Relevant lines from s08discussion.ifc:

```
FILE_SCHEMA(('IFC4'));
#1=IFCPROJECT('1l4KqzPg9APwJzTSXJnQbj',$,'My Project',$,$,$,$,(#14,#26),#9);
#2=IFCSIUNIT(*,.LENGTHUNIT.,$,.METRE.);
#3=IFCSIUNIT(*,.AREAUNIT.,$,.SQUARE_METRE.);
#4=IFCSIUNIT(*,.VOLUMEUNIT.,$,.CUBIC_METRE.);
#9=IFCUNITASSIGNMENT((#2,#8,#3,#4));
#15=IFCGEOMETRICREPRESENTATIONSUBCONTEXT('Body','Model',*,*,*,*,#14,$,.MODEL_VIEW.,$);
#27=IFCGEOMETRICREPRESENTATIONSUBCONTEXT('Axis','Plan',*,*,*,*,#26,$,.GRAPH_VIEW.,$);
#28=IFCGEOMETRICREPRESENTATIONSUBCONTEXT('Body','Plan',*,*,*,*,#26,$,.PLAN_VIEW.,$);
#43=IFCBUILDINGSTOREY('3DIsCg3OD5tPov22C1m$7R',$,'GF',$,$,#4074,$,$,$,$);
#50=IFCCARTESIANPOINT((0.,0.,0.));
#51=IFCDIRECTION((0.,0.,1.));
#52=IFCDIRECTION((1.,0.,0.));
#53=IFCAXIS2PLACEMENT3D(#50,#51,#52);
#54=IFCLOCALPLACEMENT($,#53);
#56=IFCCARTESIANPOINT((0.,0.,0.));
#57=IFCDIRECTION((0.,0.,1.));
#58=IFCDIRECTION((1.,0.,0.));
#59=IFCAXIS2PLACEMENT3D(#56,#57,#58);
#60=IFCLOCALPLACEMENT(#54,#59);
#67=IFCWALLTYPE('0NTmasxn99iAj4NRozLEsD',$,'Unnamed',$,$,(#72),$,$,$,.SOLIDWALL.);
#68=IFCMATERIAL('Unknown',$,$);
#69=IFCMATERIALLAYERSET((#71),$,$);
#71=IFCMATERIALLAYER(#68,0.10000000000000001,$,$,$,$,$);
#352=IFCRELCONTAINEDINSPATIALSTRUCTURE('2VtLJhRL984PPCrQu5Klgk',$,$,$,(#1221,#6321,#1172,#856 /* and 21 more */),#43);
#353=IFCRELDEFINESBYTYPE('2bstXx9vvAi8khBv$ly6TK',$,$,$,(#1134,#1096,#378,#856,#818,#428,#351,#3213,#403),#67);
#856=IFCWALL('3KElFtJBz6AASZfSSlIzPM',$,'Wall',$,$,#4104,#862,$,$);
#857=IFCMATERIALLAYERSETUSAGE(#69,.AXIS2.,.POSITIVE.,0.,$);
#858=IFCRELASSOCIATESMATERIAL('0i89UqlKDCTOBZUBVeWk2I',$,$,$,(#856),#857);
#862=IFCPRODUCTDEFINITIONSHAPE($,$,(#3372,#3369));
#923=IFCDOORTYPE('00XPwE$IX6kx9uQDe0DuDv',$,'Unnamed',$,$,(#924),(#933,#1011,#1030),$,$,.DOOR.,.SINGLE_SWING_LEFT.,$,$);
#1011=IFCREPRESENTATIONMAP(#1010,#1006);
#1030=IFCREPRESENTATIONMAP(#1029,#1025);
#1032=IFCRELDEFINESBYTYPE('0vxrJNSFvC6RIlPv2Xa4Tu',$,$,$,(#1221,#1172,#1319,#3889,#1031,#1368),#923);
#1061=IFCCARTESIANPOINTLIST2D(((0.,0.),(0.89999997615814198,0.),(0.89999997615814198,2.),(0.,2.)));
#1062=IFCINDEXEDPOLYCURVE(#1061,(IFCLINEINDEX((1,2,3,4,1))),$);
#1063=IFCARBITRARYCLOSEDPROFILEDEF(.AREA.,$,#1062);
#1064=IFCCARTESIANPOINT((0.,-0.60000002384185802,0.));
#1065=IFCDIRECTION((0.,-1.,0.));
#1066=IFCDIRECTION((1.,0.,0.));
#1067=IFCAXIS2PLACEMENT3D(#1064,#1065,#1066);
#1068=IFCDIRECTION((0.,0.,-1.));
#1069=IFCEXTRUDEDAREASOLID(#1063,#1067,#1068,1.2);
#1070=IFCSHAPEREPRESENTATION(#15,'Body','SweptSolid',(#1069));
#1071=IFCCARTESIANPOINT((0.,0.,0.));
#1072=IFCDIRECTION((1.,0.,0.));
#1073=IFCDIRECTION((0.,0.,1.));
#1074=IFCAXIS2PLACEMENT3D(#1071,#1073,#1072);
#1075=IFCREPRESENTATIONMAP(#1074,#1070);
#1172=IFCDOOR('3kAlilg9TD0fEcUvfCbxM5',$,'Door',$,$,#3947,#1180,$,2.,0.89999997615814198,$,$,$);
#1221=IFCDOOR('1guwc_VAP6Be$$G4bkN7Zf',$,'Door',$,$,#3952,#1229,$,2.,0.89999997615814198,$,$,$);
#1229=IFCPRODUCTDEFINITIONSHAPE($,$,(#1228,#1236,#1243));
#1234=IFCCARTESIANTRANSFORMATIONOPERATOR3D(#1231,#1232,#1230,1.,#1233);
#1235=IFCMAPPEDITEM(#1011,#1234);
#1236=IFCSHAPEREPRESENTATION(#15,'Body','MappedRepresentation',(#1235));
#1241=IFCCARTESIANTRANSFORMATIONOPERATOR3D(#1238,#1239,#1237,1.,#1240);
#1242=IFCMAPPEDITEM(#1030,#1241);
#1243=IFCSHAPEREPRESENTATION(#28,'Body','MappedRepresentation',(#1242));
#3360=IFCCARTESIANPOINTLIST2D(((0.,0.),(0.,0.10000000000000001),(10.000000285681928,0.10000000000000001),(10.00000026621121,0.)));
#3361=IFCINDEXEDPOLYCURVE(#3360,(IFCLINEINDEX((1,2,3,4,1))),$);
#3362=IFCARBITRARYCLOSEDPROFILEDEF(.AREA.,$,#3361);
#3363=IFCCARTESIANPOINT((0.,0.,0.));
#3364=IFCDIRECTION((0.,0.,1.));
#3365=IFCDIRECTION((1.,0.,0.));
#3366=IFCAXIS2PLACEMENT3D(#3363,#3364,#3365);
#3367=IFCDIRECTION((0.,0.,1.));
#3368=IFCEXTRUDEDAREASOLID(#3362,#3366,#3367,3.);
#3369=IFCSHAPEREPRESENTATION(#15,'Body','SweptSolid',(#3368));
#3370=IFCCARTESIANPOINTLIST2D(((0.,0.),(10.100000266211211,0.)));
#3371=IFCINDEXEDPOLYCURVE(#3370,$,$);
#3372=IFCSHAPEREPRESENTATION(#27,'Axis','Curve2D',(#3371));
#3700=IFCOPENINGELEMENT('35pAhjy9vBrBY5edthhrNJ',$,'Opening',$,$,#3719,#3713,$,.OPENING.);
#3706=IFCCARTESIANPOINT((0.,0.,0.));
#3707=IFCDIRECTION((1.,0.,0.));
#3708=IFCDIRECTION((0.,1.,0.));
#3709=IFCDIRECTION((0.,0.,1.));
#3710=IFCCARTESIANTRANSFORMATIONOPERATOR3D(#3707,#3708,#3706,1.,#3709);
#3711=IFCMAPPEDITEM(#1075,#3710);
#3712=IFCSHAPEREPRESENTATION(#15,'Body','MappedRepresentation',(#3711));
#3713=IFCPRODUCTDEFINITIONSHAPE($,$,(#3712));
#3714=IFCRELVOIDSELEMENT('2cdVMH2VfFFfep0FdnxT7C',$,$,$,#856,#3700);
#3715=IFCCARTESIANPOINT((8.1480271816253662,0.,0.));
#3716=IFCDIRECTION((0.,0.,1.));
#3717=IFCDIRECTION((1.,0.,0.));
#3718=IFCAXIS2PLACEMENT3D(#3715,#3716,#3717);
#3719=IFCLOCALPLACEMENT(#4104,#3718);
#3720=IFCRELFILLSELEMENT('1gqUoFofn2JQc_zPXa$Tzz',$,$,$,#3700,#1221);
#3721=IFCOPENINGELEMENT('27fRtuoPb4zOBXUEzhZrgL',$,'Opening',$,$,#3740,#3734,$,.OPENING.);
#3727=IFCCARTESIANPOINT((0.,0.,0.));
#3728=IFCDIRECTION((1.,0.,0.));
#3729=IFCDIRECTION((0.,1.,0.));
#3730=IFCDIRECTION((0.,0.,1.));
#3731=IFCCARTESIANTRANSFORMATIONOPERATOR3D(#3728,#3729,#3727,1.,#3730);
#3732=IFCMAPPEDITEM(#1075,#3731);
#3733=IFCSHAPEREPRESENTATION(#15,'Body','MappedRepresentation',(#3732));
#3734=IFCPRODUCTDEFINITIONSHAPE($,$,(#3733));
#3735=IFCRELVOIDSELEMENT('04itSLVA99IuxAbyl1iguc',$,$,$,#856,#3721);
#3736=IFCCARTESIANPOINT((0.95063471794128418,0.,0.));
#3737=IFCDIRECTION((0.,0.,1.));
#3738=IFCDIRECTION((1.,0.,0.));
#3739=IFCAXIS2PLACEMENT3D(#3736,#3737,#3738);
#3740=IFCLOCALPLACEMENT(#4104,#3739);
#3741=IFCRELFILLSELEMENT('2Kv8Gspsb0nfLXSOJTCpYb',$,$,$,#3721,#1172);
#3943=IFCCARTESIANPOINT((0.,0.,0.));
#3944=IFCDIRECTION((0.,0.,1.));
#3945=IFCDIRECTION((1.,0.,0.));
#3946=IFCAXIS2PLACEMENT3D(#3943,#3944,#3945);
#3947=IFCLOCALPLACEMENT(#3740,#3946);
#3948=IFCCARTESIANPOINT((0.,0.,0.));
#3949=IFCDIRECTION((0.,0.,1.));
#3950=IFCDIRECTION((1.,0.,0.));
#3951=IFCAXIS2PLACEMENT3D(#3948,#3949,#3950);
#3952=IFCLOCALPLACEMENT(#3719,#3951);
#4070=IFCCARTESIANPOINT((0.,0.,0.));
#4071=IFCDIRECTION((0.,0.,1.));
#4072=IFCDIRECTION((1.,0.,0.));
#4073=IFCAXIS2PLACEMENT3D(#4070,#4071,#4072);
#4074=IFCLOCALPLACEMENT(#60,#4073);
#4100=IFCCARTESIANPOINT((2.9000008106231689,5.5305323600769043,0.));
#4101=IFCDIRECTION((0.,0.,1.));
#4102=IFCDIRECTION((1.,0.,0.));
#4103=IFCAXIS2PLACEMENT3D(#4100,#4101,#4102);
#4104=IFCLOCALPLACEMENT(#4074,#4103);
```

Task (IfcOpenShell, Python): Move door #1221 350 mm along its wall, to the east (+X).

```python
import ifcopenshell
import ifcopenshell.api.geometry
import ifcopenshell.util.placement
import ifcopenshell.util.unit

model = ifcopenshell.open("s08discussion.ifc")
unit_scale = ifcopenshell.util.unit.calculate_unit_scale(model)

door = model.by_guid("1guwc_VAP6Be$$G4bkN7Zf")
opening = door.FillsVoids[0].RelatingOpeningElement
wall = opening.VoidsElements[0].RelatingBuildingElement

wall_matrix = ifcopenshell.util.placement.get_local_placement(wall.ObjectPlacement)
shift = wall_matrix[:3, 0] * 0.35 / unit_scale
before = ifcopenshell.util.placement.get_local_placement(door.ObjectPlacement)[:3, 3].copy()

# The door is placed relative to its opening, so it follows when the opening moves.
matrix = ifcopenshell.util.placement.get_local_placement(opening.ObjectPlacement)
matrix[:3, 3] += shift
ifcopenshell.api.geometry.edit_object_placement(
    model, product=opening, matrix=matrix, is_si=False, should_transform_children=True
)

after = ifcopenshell.util.placement.get_local_placement(door.ObjectPlacement)[:3, 3]
print("door moved by", (after - before).round(3) + 0.0)

model.write("s08discussion_rev.ifc")
```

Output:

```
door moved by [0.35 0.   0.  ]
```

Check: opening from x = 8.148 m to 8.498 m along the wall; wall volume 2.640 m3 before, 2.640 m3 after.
